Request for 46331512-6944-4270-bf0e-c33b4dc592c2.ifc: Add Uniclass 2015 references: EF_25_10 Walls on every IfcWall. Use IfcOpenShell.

First a look at what the model holds.

```python
import ifcopenshell

model = ifcopenshell.open("46331512-6944-4270-bf0e-c33b4dc592c2.ifc")
print(model.schema)
print("classifications:", [c.Name for c in model.by_type("IfcClassification")])
for ifc_class in ("IfcDoor", "IfcRoof", "IfcStair", "IfcWall", "IfcWindow"):
    print(ifc_class, len(model.by_type(ifc_class)))
```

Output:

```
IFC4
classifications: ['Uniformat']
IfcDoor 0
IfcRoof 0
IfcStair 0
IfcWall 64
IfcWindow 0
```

```python
import ifcopenshell
import ifcopenshell.api.classification

model = ifcopenshell.open("46331512-6944-4270-bf0e-c33b4dc592c2.ifc")

system = ifcopenshell.api.classification.add_classification(model, classification="Uniclass 2015")

codes = {
    "IfcWall": ("EF_25_10", "Walls"),
}
for ifc_class, (code, name) in codes.items():
    products = model.by_type(ifc_class)
    ifcopenshell.api.classification.add_reference(
        model, products=products, classification=system, identification=code, name=name
    )
    print(code, len(products))

model.write("46331512-6944-4270-bf0e-c33b4dc592c2_updated.ifc")
```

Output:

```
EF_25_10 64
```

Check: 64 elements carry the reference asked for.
